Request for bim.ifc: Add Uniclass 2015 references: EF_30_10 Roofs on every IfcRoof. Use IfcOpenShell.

First a look at what the model holds.

```python
import ifcopenshell

model = ifcopenshell.open("bim.ifc")
print(model.schema)
print("classifications:", [c.Name for c in model.by_type("IfcClassification")])
for ifc_class in ("IfcDoor", "IfcRoof", "IfcStair", "IfcWall", "IfcWindow"):
    print(ifc_class, len(model.by_type(ifc_class)))
```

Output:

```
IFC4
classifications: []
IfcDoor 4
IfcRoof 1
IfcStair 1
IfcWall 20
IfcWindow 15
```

```python
import ifcopenshell
import ifcopenshell.api.classification

model = ifcopenshell.open("bim.ifc")

system = ifcopenshell.api.classification.add_classification(model, classification="Uniclass 2015")

codes = {
    "IfcRoof": ("EF_30_10", "Roofs"),
}
for ifc_class, (code, name) in codes.items():
    products = model.by_type(ifc_class)
    ifcopenshell.api.classification.add_reference(
        model, products=products, classification=system, identification=code, name=name
    )
    print(code, len(products))

model.write("bim_edited.ifc")
```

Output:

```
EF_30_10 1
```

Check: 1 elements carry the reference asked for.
